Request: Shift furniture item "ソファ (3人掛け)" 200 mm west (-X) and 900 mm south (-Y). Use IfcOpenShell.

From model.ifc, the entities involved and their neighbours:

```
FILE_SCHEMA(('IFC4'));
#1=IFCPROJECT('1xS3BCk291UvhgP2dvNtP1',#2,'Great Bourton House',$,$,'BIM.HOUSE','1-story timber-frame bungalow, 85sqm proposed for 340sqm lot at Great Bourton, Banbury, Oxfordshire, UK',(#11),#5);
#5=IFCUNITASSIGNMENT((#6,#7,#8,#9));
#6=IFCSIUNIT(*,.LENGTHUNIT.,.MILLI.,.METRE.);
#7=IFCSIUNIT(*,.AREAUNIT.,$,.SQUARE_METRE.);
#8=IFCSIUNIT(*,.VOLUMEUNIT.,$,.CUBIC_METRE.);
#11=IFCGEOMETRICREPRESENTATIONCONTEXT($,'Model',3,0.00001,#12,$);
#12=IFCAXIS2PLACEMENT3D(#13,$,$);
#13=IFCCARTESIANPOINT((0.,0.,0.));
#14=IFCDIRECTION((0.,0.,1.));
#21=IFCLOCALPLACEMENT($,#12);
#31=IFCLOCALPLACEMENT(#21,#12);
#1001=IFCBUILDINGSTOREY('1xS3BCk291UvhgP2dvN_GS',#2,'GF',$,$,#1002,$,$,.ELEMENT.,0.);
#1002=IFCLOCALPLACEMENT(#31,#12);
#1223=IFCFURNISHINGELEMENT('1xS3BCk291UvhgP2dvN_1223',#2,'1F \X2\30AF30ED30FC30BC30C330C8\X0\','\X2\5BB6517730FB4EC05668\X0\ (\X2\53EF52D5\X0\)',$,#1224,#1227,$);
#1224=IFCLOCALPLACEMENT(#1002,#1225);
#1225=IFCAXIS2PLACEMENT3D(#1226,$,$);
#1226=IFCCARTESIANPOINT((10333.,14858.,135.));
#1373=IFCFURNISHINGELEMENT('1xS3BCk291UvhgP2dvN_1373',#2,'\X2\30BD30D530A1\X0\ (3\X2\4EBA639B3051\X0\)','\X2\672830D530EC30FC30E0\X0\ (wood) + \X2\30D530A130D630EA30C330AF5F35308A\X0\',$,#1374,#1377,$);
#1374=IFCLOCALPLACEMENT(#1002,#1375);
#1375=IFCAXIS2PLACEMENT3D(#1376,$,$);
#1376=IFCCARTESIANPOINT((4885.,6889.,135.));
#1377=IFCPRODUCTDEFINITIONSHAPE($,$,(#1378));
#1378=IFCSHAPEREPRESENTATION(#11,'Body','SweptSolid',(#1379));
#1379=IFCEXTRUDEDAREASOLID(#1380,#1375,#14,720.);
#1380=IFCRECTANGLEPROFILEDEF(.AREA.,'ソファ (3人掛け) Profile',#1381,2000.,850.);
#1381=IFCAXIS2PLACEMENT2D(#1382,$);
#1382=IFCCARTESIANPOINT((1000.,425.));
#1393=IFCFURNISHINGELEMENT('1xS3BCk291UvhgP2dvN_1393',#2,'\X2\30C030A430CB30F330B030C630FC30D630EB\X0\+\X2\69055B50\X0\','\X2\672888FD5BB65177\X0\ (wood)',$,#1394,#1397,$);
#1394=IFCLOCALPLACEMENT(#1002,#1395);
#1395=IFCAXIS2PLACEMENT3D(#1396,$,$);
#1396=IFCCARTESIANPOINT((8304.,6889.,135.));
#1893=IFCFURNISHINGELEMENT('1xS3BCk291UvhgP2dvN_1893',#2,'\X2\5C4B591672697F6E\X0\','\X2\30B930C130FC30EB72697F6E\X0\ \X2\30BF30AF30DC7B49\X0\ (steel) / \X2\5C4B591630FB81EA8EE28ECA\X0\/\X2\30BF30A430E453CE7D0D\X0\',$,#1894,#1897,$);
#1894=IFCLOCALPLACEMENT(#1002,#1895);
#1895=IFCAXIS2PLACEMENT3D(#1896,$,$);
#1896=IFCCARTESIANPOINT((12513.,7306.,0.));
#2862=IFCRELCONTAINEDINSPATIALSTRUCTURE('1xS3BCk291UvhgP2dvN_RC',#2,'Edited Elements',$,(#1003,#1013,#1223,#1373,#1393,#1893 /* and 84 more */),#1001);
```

```python
import ifcopenshell
import ifcopenshell.api.geometry
import ifcopenshell.util.placement
import ifcopenshell.util.unit

model = ifcopenshell.open("model.ifc")
unit_scale = ifcopenshell.util.unit.calculate_unit_scale(model)

item = model.by_guid("1xS3BCk291UvhgP2dvN_1373")
matrix = ifcopenshell.util.placement.get_local_placement(item.ObjectPlacement)
matrix[0, 3] -= 0.2 / unit_scale
matrix[1, 3] -= 0.9 / unit_scale
ifcopenshell.api.geometry.edit_object_placement(model, product=item, matrix=matrix, is_si=False)

print(ifcopenshell.util.placement.get_local_placement(item.ObjectPlacement).round(3) + 0.0)

model.write("model_rev.ifc")
```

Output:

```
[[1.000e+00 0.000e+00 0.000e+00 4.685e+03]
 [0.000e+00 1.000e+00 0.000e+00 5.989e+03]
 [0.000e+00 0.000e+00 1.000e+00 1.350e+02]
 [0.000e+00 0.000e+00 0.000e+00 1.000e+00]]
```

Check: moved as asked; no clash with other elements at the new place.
